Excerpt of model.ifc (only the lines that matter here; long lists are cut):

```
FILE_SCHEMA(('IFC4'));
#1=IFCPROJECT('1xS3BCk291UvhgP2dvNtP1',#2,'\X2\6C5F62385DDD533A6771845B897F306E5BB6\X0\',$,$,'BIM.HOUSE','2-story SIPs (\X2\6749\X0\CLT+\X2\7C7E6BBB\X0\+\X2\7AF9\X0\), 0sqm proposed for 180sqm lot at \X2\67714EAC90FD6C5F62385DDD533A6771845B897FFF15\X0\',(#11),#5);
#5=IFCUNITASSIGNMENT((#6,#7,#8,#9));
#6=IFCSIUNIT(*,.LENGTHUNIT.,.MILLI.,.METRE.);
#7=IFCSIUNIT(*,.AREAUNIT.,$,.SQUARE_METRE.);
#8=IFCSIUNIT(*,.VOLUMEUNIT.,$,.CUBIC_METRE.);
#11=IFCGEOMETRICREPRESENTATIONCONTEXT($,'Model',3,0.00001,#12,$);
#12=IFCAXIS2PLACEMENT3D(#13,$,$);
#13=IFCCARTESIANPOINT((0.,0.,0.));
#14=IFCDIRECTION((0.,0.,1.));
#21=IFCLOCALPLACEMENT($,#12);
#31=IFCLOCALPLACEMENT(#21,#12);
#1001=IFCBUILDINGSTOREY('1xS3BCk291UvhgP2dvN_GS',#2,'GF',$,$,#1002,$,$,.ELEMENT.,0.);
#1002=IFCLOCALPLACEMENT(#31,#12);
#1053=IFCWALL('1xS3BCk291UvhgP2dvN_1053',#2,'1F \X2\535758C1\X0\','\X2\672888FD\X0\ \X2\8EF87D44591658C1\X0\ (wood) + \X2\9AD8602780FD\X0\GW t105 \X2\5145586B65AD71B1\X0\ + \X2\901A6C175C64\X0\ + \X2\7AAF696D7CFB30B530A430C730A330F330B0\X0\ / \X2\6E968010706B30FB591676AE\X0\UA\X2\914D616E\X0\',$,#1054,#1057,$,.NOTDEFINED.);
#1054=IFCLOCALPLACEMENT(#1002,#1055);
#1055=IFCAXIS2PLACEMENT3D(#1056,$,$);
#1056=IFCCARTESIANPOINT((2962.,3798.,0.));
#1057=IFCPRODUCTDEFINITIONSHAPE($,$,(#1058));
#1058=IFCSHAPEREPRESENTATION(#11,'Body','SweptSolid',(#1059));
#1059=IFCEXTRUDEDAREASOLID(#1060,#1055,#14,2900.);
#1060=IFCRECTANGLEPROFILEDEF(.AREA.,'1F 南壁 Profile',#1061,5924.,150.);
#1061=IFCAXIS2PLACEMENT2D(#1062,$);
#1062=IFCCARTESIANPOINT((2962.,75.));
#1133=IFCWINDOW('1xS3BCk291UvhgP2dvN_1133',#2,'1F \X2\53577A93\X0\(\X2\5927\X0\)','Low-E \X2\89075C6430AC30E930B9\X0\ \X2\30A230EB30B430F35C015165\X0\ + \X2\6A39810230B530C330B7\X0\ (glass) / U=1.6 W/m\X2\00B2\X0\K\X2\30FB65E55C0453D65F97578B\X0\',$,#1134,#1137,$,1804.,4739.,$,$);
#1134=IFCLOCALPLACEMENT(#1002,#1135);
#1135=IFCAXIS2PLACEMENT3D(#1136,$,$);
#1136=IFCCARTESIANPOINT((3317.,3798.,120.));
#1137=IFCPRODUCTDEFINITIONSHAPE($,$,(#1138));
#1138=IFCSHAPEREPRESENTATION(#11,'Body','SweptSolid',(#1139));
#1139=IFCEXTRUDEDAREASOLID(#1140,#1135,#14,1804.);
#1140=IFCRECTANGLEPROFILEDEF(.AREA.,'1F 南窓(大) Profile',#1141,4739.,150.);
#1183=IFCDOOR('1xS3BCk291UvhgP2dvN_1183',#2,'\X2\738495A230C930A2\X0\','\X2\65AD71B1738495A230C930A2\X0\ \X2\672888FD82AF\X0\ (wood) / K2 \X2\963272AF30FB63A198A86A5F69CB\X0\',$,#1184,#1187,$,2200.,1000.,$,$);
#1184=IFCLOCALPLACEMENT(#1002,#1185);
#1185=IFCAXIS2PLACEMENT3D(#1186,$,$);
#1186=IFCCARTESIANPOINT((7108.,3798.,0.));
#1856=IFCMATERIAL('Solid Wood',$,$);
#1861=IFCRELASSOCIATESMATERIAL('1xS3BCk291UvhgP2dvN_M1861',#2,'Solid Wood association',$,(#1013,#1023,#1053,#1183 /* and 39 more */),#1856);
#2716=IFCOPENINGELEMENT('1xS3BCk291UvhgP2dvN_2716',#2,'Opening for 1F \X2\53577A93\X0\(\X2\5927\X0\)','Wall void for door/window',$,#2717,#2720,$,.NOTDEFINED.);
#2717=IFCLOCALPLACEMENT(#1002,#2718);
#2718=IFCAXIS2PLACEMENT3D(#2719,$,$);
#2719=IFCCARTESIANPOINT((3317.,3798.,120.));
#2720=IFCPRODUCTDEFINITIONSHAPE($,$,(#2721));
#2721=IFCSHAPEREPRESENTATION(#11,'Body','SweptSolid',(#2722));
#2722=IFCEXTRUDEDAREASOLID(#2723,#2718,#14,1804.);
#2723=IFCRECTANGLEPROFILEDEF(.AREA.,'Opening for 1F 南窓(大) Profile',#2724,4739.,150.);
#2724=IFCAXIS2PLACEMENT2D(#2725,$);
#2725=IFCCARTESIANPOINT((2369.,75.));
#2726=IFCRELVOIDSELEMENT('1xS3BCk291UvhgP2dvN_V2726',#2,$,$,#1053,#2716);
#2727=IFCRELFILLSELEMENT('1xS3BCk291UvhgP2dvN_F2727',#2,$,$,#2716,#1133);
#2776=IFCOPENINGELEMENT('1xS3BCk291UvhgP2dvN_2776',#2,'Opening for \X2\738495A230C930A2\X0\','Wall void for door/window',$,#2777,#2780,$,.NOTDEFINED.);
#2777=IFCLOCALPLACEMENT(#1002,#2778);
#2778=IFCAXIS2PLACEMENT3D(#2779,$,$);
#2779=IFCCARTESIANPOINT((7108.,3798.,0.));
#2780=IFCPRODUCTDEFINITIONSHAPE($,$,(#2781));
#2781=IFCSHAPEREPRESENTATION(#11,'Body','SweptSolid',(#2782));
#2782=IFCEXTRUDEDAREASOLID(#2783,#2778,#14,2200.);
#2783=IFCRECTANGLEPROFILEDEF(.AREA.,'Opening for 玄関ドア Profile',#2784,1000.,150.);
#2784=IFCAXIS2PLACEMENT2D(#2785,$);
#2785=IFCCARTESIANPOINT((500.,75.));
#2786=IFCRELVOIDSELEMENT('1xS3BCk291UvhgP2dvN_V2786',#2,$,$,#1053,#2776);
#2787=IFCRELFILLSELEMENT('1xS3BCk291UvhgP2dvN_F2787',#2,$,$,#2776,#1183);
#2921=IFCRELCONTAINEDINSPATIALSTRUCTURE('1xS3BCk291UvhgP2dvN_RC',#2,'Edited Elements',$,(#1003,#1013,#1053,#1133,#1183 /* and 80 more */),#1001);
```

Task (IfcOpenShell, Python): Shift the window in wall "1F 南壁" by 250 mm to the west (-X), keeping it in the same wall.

```python
import ifcopenshell
import ifcopenshell.api.geometry
import ifcopenshell.util.placement

model = ifcopenshell.open("model.ifc")

window = model.by_id(1133)
opening = window.FillsVoids[0].RelatingOpeningElement
wall = opening.VoidsElements[0].RelatingBuildingElement

wall_matrix = ifcopenshell.util.placement.get_local_placement(wall.ObjectPlacement)
shift = wall_matrix[:3, 0] * -250.0
before = ifcopenshell.util.placement.get_local_placement(window.ObjectPlacement)[:3, 3].copy()

# The window is not placed relative to its opening, so move both.
for product in (opening, window):
    matrix = ifcopenshell.util.placement.get_local_placement(product.ObjectPlacement)
    matrix[:3, 3] += shift
    ifcopenshell.api.geometry.edit_object_placement(model, product=product, matrix=matrix, is_si=False)

after = ifcopenshell.util.placement.get_local_placement(window.ObjectPlacement)[:3, 3]
print("window moved by", (after - before).round(3) + 0.0)

model.write("model_v2.ifc")
```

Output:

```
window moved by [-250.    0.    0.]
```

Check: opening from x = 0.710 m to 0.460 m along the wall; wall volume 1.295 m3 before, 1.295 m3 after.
